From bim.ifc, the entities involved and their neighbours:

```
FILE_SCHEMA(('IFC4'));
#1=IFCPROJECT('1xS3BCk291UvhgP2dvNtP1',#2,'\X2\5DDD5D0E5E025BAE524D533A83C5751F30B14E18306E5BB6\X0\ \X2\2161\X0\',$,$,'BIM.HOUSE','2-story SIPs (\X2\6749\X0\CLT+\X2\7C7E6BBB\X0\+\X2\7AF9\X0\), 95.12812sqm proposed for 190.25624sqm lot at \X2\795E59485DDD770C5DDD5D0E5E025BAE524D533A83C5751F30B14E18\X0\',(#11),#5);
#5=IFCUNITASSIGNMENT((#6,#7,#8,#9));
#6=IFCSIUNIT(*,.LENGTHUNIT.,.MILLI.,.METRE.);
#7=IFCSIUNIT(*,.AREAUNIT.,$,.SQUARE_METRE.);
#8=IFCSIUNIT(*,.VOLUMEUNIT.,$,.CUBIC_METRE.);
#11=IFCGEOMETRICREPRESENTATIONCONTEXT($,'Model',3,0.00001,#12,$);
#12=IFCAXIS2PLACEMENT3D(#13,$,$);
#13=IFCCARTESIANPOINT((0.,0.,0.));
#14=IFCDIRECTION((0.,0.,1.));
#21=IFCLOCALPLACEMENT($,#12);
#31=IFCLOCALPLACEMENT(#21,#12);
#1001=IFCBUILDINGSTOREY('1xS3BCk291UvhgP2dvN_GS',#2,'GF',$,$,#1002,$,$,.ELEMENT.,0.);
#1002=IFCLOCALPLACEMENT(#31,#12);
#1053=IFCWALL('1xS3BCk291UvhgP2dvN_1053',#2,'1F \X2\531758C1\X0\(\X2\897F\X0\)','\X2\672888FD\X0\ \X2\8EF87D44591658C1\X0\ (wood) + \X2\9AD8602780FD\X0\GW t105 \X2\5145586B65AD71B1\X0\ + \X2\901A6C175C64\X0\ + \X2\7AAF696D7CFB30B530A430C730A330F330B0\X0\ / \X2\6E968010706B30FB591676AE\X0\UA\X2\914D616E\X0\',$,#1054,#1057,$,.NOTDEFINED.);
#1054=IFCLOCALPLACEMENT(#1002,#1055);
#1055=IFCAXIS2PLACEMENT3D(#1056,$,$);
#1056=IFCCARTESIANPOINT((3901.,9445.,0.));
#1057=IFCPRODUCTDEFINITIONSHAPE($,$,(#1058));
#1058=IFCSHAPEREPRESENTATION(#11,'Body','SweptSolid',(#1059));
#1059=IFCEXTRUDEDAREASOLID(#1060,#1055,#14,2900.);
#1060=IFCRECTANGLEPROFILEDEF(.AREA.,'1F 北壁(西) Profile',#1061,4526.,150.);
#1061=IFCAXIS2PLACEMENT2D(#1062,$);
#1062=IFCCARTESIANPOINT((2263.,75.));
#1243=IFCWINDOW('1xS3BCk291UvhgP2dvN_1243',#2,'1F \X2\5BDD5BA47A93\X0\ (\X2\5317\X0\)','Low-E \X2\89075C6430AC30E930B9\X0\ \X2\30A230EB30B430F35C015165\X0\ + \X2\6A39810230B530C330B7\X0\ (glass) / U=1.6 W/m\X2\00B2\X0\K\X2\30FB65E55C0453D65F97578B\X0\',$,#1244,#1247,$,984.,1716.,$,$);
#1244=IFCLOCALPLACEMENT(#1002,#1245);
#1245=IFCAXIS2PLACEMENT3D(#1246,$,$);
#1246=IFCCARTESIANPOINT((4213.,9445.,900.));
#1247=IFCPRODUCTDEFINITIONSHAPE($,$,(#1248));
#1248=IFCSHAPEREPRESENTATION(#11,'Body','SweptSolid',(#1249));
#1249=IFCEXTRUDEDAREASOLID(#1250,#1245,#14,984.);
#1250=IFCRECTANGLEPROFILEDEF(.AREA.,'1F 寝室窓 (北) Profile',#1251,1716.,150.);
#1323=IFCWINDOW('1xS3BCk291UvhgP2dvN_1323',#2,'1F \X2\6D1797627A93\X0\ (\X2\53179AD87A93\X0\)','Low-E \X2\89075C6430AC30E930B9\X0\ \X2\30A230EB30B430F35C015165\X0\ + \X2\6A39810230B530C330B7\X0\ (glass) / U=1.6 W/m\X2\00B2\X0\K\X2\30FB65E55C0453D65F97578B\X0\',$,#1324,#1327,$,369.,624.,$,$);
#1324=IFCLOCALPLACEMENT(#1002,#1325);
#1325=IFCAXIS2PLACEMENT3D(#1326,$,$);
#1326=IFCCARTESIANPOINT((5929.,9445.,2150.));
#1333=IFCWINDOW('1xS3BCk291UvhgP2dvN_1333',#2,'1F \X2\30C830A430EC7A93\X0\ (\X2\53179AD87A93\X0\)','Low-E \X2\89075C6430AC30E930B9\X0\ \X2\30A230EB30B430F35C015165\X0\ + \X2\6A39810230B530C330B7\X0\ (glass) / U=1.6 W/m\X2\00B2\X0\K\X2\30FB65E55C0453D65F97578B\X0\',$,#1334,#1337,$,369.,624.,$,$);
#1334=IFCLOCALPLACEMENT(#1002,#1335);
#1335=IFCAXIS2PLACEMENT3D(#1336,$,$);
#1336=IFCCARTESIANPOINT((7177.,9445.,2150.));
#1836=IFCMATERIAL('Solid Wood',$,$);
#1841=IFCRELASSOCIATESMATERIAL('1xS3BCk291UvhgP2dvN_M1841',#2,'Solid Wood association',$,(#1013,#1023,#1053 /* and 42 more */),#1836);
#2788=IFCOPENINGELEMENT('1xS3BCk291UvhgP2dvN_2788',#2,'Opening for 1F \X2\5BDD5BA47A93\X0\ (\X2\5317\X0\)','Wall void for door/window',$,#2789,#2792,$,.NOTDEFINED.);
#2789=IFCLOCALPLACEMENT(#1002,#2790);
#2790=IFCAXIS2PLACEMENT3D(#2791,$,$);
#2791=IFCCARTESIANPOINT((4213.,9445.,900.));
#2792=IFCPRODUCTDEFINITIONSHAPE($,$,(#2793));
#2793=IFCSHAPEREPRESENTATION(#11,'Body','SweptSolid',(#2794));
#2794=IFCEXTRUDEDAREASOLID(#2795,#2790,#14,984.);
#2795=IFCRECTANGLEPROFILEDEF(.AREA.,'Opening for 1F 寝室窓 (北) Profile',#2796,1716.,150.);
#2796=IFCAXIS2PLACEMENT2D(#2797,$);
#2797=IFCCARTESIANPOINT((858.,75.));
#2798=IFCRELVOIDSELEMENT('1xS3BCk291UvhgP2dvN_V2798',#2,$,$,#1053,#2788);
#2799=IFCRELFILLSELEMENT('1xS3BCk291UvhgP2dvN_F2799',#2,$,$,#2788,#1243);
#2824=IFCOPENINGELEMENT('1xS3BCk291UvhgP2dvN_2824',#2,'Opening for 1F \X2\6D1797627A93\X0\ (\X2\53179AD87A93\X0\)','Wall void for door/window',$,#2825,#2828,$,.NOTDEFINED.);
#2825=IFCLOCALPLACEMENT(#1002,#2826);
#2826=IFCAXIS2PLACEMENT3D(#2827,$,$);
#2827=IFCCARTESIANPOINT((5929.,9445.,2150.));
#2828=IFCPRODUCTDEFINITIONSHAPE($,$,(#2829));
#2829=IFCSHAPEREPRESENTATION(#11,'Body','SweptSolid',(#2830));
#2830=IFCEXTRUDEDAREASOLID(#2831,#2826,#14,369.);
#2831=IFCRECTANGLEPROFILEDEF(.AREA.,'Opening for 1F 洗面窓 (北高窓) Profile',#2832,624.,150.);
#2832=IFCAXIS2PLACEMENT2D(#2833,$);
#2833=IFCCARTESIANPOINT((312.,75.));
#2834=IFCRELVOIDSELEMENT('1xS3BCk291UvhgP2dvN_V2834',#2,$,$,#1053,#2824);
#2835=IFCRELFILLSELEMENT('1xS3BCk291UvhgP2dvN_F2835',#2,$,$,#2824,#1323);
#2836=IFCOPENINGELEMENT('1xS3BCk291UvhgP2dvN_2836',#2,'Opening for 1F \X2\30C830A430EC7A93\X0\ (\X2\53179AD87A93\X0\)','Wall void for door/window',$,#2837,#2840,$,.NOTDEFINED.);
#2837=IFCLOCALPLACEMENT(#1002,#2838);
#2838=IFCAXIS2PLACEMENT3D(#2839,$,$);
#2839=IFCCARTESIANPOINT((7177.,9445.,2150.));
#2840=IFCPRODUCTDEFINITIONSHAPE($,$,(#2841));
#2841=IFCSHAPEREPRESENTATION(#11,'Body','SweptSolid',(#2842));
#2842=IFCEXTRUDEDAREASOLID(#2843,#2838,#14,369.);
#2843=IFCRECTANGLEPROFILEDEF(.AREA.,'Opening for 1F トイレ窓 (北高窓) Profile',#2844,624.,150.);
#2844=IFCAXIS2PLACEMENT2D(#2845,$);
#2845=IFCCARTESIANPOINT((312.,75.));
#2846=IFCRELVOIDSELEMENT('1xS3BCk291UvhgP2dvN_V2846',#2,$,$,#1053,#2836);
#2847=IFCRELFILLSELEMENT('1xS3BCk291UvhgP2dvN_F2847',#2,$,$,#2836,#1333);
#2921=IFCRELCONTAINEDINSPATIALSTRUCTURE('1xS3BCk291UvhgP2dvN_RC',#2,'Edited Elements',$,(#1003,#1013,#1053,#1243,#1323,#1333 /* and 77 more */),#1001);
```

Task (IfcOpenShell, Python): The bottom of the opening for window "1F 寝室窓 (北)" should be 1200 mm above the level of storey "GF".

```python
import numpy as np
import ifcopenshell
import ifcopenshell.api.geometry
import ifcopenshell.geom
import ifcopenshell.util.element
import ifcopenshell.util.placement
import ifcopenshell.util.shape
import ifcopenshell.util.unit

model = ifcopenshell.open("bim.ifc")
unit_scale = ifcopenshell.util.unit.calculate_unit_scale(model)

window = model.by_guid("1xS3BCk291UvhgP2dvN_1243")
opening = window.FillsVoids[0].RelatingOpeningElement
storey = ifcopenshell.util.element.get_container(window, ifc_class="IfcBuildingStorey")
level = ifcopenshell.util.placement.get_local_placement(storey.ObjectPlacement)[2, 3]

# The opening's origin need not be at the sill, so measure its lowest point.
shape = ifcopenshell.geom.create_shape(ifcopenshell.geom.settings(), opening)
bottom = ifcopenshell.util.shape.get_shape_bottom_elevation(shape, shape.geometry) / unit_scale
dz = level + 1.2 / unit_scale - bottom

shift = np.array([0.0, 0.0, dz])
# The window is not placed relative to its opening, so move both.
for product in (opening, window):
    matrix = ifcopenshell.util.placement.get_local_placement(product.ObjectPlacement)
    matrix[:3, 3] += shift
    ifcopenshell.api.geometry.edit_object_placement(model, product=product, matrix=matrix, is_si=False)

print(f"moved by {dz * unit_scale:+.3f} m")

model.write("bim_updated.ifc")
```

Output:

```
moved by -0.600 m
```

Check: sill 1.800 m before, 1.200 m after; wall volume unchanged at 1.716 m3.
